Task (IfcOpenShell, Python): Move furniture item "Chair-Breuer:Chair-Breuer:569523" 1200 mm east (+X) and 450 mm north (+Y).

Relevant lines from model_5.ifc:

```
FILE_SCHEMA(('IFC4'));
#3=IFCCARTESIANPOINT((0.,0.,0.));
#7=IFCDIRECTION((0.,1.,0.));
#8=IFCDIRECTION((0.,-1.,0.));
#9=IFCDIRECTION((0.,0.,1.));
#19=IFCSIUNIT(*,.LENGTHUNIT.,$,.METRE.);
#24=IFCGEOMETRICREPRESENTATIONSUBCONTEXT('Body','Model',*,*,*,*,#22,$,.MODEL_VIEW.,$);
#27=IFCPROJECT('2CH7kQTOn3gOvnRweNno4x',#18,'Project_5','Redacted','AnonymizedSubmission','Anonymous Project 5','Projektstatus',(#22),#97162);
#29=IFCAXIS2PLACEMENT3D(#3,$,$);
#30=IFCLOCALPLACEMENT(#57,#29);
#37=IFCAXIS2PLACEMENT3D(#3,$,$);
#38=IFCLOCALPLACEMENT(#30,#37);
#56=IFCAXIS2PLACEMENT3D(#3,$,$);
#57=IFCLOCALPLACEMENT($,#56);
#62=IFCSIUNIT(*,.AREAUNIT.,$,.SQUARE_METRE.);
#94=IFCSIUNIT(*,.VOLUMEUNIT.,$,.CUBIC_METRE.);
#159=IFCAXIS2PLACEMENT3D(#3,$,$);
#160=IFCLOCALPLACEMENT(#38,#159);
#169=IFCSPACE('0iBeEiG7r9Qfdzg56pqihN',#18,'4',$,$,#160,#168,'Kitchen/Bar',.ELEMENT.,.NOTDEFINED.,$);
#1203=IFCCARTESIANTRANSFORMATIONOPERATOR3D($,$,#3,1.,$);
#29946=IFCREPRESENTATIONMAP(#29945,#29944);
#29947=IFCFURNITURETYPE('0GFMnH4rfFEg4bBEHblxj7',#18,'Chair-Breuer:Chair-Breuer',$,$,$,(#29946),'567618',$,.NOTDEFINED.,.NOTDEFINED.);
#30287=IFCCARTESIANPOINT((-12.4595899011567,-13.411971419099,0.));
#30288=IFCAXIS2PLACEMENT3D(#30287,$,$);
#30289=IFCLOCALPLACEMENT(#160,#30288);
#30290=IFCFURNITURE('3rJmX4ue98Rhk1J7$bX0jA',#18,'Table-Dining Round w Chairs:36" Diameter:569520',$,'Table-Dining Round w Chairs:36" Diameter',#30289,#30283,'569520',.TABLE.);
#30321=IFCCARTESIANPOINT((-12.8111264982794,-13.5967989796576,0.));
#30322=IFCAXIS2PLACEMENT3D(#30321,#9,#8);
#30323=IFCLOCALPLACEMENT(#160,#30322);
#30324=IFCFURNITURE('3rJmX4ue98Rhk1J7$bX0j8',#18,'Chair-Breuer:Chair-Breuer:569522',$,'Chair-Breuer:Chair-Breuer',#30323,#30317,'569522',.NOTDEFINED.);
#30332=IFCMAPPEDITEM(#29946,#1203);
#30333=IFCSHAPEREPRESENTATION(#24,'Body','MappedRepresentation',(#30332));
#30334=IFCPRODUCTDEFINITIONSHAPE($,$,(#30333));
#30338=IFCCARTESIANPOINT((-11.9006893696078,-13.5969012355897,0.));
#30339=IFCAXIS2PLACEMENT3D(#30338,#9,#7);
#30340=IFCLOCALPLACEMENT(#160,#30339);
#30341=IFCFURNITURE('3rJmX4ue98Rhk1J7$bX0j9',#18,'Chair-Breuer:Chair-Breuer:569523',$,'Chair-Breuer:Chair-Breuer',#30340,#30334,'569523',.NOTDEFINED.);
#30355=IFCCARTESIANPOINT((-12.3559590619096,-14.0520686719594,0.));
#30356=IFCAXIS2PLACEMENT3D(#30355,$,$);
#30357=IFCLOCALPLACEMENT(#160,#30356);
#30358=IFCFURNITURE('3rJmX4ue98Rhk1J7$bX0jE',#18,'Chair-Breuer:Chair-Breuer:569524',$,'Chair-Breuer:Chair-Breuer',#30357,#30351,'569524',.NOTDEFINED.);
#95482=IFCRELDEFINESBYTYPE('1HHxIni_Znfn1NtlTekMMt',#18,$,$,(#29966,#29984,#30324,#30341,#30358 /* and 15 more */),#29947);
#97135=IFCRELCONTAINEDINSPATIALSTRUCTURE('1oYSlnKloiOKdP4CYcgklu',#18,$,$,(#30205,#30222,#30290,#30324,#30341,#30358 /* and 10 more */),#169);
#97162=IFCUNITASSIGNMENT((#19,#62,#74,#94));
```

```python
import ifcopenshell
import ifcopenshell.api.geometry
import ifcopenshell.util.placement
import ifcopenshell.util.unit

model = ifcopenshell.open("model_5.ifc")
unit_scale = ifcopenshell.util.unit.calculate_unit_scale(model)

item = model.by_id(30341)
matrix = ifcopenshell.util.placement.get_local_placement(item.ObjectPlacement)
matrix[0, 3] += 1.2 / unit_scale
matrix[1, 3] += 0.45 / unit_scale
ifcopenshell.api.geometry.edit_object_placement(model, product=item, matrix=matrix, is_si=False)

print(ifcopenshell.util.placement.get_local_placement(item.ObjectPlacement).round(3) + 0.0)

model.write("model_5-out.ifc")
```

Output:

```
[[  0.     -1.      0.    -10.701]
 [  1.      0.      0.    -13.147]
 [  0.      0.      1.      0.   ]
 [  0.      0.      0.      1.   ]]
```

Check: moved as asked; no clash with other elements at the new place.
